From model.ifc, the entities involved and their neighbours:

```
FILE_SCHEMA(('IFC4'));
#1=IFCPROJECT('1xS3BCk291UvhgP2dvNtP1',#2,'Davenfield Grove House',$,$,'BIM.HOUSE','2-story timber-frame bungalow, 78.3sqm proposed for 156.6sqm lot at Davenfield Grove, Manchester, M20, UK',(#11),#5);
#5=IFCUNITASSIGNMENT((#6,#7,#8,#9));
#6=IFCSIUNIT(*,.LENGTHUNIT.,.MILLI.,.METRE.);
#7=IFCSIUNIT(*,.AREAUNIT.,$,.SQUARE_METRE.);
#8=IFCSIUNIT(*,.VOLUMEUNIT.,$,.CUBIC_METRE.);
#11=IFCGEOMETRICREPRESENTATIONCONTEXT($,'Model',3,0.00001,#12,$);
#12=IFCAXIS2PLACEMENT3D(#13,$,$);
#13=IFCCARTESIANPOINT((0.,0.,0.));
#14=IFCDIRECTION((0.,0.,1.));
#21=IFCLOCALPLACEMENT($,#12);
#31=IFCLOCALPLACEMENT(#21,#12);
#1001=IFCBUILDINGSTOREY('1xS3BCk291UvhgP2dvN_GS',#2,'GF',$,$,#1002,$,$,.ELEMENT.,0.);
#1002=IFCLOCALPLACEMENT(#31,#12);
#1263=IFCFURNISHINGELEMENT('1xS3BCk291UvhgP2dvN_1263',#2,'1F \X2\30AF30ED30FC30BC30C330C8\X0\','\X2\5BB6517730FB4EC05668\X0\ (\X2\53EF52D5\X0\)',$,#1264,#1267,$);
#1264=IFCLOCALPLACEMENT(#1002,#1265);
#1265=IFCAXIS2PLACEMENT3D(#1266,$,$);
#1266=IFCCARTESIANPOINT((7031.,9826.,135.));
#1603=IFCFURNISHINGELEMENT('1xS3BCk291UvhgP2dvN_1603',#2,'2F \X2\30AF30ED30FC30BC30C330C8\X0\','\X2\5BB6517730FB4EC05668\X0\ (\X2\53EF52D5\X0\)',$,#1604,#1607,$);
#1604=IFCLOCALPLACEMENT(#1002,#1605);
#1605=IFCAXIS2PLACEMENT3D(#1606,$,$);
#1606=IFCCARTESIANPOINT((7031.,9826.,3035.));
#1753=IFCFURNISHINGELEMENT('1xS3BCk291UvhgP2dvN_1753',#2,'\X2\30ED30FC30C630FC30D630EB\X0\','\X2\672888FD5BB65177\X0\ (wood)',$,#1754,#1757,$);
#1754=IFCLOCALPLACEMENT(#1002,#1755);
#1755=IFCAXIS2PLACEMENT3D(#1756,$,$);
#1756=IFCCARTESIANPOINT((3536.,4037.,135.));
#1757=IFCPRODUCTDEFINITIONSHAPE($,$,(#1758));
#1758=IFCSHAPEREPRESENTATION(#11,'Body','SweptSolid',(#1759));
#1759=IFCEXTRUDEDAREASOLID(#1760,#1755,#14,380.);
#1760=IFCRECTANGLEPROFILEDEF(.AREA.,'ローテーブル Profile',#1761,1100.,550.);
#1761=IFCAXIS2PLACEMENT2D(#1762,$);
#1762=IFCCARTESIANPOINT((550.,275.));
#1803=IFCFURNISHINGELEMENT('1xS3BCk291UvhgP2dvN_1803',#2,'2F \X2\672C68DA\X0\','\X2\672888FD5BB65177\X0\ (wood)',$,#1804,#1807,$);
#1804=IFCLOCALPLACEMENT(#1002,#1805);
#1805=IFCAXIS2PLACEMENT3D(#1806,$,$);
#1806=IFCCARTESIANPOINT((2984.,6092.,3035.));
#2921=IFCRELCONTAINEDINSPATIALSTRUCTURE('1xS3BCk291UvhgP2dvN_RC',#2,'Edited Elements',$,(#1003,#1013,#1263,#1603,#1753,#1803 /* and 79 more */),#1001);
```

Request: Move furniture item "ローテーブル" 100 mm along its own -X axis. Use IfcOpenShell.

```python
import ifcopenshell
import ifcopenshell.api.geometry
import ifcopenshell.util.placement

model = ifcopenshell.open("model.ifc")

item = model.by_guid("1xS3BCk291UvhgP2dvN_1753")
matrix = ifcopenshell.util.placement.get_local_placement(item.ObjectPlacement)
matrix[:3, 3] -= matrix[:3, 0] * 100.0
ifcopenshell.api.geometry.edit_object_placement(model, product=item, matrix=matrix, is_si=False)

print(ifcopenshell.util.placement.get_local_placement(item.ObjectPlacement).round(3) + 0.0)

model.write("model_v2.ifc")
```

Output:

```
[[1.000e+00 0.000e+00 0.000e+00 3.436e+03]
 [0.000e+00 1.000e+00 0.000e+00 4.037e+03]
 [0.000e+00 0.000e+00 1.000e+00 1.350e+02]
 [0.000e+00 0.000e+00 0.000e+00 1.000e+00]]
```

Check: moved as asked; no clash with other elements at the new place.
